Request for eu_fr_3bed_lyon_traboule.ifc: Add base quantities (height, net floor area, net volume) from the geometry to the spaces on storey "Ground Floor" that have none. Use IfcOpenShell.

First a look at what the model holds.

```python
import ifcopenshell
import ifcopenshell.util.element
import ifcopenshell.util.unit

model = ifcopenshell.open("eu_fr_3bed_lyon_traboule.ifc")
print(model.schema)
for unit_type in ("LENGTHUNIT", "AREAUNIT", "VOLUMEUNIT"):
    print(unit_type, ifcopenshell.util.unit.calculate_unit_scale(model, unit_type))
storey = next(s for s in model.by_type("IfcBuildingStorey") if s.Name == "Ground Floor")
spaces = [e for e in ifcopenshell.util.element.get_decomposition(storey) if e.is_a("IfcSpace")]
for e in sorted(spaces, key=lambda e: e.id()):
    print(e.id(), e.is_a(), e.Name, list(ifcopenshell.util.element.get_psets(e, qtos_only=True)), sep=" | ")
```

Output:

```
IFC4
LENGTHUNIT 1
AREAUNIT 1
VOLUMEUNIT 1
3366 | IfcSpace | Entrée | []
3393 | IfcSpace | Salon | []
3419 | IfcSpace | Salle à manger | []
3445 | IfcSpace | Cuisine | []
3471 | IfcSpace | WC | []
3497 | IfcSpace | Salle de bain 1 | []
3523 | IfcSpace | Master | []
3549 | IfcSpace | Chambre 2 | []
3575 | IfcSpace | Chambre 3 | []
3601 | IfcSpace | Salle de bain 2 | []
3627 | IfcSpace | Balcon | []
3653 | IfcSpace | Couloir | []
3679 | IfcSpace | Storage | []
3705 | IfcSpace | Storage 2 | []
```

```python
import ifcopenshell
import ifcopenshell.api.pset
import ifcopenshell.geom
import ifcopenshell.util.element
import ifcopenshell.util.shape
import ifcopenshell.util.unit

model = ifcopenshell.open("eu_fr_3bed_lyon_traboule.ifc")
unit_scale = ifcopenshell.util.unit.calculate_unit_scale(model)
area_scale = ifcopenshell.util.unit.calculate_unit_scale(model, "AREAUNIT")
volume_scale = ifcopenshell.util.unit.calculate_unit_scale(model, "VOLUMEUNIT")
settings = ifcopenshell.geom.settings()

storey = next(s for s in model.by_type("IfcBuildingStorey") if s.Name == "Ground Floor")
spaces = [e for e in ifcopenshell.util.element.get_decomposition(storey) if e.is_a("IfcSpace")]

for e in sorted(spaces, key=lambda e: e.id()):
    if ifcopenshell.util.element.get_psets(e, qtos_only=True, should_inherit=False):
        continue
    # Geometry comes back in metres, in the element's own axes.
    shape = ifcopenshell.geom.create_shape(settings, e)
    values = {
        "Height": ifcopenshell.util.shape.get_z(shape.geometry) / unit_scale,
        "NetFloorArea": ifcopenshell.util.shape.get_footprint_area(shape.geometry) / area_scale,
        "NetVolume": ifcopenshell.util.shape.get_volume(shape.geometry) / volume_scale,
    }
    qto = ifcopenshell.api.pset.add_qto(model, product=e, name="Qto_SpaceBaseQuantities")
    ifcopenshell.api.pset.edit_qto(model, qto=qto, properties=values)
    print(e.id(), {k: round(v, 3) for k, v in values.items()})

model.write("eu_fr_3bed_lyon_traboule_edited.ifc")
```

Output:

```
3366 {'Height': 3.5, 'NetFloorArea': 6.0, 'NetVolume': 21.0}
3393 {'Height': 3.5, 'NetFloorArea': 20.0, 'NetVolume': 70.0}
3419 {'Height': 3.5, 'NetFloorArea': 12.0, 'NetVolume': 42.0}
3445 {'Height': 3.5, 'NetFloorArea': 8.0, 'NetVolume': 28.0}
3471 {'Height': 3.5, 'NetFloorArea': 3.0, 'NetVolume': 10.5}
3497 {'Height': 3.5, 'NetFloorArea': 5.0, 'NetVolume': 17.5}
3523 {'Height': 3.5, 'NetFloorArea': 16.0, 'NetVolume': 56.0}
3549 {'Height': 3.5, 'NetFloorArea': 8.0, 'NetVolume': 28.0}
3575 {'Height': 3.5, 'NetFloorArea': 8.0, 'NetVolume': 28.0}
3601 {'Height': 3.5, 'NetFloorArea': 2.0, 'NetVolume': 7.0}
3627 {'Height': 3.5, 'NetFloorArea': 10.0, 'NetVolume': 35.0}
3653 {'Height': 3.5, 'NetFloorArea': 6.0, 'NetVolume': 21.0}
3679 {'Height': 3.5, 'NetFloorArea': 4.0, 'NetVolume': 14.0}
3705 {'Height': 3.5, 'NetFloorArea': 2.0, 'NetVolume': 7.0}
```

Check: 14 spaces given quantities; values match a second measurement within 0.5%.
